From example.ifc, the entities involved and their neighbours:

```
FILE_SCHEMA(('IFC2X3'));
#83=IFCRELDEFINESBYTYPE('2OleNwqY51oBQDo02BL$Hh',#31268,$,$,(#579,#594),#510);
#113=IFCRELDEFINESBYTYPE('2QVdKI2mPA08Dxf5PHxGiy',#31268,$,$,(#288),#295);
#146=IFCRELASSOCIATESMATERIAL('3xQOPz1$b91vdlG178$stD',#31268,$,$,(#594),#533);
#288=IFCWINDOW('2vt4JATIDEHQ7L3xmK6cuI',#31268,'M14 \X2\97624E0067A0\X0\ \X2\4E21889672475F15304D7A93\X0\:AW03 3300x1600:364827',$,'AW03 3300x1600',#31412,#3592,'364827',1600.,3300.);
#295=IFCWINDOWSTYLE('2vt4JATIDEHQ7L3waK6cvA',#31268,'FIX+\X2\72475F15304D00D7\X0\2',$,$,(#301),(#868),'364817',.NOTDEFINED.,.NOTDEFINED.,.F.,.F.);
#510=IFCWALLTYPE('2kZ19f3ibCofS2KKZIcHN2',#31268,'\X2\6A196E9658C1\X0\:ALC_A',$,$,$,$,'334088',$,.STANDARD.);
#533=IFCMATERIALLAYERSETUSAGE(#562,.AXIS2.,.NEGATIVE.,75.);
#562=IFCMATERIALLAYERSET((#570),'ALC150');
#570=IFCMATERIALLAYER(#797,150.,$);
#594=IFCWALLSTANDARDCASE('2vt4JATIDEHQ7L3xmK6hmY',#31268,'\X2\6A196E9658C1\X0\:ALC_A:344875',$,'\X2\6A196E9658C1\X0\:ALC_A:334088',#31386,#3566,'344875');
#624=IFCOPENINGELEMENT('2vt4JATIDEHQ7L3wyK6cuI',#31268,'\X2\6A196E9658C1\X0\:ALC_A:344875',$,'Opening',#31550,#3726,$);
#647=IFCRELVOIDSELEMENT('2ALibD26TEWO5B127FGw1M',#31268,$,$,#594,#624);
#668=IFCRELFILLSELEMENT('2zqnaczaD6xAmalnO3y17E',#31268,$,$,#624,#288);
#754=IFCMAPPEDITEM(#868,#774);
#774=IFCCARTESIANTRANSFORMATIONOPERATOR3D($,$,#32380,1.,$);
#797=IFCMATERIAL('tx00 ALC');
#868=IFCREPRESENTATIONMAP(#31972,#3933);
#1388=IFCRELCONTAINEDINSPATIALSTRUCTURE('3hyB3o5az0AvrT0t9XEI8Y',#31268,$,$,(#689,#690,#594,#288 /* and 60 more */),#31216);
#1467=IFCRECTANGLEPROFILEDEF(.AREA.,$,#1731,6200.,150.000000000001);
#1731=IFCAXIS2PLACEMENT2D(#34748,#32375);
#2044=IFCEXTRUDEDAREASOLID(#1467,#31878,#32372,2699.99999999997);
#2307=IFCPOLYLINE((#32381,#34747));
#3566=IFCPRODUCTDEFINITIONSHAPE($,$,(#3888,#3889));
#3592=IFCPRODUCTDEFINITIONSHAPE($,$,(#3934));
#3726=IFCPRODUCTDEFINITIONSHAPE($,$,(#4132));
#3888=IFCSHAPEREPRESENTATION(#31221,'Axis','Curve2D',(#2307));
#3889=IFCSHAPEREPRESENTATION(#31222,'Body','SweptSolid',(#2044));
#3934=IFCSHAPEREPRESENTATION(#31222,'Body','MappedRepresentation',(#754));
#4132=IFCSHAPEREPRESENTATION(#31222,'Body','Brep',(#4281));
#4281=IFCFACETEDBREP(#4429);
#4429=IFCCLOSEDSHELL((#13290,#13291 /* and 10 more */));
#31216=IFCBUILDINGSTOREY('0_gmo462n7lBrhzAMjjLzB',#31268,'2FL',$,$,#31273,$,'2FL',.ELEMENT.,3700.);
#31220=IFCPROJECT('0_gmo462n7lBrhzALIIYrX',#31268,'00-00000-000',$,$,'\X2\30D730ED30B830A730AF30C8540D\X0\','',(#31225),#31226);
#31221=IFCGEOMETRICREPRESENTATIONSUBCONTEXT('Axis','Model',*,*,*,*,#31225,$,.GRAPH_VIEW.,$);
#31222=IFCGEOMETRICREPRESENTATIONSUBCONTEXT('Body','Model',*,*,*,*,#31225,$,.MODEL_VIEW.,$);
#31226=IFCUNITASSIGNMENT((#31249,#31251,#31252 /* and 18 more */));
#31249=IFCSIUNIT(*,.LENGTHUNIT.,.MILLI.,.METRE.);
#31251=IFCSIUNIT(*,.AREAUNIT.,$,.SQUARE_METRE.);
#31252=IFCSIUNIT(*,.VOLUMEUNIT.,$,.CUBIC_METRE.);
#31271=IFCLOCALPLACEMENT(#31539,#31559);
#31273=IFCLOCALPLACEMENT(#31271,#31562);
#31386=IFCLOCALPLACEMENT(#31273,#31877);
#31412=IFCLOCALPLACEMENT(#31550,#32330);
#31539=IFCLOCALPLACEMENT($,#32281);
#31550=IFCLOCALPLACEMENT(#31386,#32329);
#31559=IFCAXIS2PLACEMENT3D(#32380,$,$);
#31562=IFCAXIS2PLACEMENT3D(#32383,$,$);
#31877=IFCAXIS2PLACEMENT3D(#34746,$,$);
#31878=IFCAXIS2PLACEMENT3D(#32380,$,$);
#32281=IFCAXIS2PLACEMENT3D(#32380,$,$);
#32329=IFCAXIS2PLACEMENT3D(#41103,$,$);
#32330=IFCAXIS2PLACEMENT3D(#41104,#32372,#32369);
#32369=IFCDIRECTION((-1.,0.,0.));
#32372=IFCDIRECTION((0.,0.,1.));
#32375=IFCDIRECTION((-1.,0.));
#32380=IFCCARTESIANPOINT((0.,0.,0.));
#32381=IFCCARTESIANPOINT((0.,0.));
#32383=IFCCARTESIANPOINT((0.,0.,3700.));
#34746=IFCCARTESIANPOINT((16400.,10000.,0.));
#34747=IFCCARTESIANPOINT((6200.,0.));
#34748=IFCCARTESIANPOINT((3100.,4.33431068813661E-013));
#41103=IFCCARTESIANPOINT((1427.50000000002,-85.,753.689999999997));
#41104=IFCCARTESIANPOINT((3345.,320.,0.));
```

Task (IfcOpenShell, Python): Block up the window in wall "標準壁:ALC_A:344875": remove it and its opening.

```python
import ifcopenshell
import ifcopenshell.api.feature
import ifcopenshell.api.root
import ifcopenshell.geom
import ifcopenshell.util.shape

model = ifcopenshell.open("example.ifc")
settings = ifcopenshell.geom.settings()


def volume(element):
    """Net volume in cubic metres, openings subtracted."""
    shape = ifcopenshell.geom.create_shape(settings, element)
    return ifcopenshell.util.shape.get_volume(shape.geometry)


window = model.by_guid("2vt4JATIDEHQ7L3xmK6cuI")
opening = window.FillsVoids[0].RelatingOpeningElement
wall = opening.VoidsElements[0].RelatingBuildingElement
before = volume(wall)

ifcopenshell.api.root.remove_product(model, product=window)
ifcopenshell.api.feature.remove_feature(model, feature=opening)

after = volume(wall)

print(f"wall volume {before:.3f} -> {after:.3f} m3")

model.write("example-out.ifc")
```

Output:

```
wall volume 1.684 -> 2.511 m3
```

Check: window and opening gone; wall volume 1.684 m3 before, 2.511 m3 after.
